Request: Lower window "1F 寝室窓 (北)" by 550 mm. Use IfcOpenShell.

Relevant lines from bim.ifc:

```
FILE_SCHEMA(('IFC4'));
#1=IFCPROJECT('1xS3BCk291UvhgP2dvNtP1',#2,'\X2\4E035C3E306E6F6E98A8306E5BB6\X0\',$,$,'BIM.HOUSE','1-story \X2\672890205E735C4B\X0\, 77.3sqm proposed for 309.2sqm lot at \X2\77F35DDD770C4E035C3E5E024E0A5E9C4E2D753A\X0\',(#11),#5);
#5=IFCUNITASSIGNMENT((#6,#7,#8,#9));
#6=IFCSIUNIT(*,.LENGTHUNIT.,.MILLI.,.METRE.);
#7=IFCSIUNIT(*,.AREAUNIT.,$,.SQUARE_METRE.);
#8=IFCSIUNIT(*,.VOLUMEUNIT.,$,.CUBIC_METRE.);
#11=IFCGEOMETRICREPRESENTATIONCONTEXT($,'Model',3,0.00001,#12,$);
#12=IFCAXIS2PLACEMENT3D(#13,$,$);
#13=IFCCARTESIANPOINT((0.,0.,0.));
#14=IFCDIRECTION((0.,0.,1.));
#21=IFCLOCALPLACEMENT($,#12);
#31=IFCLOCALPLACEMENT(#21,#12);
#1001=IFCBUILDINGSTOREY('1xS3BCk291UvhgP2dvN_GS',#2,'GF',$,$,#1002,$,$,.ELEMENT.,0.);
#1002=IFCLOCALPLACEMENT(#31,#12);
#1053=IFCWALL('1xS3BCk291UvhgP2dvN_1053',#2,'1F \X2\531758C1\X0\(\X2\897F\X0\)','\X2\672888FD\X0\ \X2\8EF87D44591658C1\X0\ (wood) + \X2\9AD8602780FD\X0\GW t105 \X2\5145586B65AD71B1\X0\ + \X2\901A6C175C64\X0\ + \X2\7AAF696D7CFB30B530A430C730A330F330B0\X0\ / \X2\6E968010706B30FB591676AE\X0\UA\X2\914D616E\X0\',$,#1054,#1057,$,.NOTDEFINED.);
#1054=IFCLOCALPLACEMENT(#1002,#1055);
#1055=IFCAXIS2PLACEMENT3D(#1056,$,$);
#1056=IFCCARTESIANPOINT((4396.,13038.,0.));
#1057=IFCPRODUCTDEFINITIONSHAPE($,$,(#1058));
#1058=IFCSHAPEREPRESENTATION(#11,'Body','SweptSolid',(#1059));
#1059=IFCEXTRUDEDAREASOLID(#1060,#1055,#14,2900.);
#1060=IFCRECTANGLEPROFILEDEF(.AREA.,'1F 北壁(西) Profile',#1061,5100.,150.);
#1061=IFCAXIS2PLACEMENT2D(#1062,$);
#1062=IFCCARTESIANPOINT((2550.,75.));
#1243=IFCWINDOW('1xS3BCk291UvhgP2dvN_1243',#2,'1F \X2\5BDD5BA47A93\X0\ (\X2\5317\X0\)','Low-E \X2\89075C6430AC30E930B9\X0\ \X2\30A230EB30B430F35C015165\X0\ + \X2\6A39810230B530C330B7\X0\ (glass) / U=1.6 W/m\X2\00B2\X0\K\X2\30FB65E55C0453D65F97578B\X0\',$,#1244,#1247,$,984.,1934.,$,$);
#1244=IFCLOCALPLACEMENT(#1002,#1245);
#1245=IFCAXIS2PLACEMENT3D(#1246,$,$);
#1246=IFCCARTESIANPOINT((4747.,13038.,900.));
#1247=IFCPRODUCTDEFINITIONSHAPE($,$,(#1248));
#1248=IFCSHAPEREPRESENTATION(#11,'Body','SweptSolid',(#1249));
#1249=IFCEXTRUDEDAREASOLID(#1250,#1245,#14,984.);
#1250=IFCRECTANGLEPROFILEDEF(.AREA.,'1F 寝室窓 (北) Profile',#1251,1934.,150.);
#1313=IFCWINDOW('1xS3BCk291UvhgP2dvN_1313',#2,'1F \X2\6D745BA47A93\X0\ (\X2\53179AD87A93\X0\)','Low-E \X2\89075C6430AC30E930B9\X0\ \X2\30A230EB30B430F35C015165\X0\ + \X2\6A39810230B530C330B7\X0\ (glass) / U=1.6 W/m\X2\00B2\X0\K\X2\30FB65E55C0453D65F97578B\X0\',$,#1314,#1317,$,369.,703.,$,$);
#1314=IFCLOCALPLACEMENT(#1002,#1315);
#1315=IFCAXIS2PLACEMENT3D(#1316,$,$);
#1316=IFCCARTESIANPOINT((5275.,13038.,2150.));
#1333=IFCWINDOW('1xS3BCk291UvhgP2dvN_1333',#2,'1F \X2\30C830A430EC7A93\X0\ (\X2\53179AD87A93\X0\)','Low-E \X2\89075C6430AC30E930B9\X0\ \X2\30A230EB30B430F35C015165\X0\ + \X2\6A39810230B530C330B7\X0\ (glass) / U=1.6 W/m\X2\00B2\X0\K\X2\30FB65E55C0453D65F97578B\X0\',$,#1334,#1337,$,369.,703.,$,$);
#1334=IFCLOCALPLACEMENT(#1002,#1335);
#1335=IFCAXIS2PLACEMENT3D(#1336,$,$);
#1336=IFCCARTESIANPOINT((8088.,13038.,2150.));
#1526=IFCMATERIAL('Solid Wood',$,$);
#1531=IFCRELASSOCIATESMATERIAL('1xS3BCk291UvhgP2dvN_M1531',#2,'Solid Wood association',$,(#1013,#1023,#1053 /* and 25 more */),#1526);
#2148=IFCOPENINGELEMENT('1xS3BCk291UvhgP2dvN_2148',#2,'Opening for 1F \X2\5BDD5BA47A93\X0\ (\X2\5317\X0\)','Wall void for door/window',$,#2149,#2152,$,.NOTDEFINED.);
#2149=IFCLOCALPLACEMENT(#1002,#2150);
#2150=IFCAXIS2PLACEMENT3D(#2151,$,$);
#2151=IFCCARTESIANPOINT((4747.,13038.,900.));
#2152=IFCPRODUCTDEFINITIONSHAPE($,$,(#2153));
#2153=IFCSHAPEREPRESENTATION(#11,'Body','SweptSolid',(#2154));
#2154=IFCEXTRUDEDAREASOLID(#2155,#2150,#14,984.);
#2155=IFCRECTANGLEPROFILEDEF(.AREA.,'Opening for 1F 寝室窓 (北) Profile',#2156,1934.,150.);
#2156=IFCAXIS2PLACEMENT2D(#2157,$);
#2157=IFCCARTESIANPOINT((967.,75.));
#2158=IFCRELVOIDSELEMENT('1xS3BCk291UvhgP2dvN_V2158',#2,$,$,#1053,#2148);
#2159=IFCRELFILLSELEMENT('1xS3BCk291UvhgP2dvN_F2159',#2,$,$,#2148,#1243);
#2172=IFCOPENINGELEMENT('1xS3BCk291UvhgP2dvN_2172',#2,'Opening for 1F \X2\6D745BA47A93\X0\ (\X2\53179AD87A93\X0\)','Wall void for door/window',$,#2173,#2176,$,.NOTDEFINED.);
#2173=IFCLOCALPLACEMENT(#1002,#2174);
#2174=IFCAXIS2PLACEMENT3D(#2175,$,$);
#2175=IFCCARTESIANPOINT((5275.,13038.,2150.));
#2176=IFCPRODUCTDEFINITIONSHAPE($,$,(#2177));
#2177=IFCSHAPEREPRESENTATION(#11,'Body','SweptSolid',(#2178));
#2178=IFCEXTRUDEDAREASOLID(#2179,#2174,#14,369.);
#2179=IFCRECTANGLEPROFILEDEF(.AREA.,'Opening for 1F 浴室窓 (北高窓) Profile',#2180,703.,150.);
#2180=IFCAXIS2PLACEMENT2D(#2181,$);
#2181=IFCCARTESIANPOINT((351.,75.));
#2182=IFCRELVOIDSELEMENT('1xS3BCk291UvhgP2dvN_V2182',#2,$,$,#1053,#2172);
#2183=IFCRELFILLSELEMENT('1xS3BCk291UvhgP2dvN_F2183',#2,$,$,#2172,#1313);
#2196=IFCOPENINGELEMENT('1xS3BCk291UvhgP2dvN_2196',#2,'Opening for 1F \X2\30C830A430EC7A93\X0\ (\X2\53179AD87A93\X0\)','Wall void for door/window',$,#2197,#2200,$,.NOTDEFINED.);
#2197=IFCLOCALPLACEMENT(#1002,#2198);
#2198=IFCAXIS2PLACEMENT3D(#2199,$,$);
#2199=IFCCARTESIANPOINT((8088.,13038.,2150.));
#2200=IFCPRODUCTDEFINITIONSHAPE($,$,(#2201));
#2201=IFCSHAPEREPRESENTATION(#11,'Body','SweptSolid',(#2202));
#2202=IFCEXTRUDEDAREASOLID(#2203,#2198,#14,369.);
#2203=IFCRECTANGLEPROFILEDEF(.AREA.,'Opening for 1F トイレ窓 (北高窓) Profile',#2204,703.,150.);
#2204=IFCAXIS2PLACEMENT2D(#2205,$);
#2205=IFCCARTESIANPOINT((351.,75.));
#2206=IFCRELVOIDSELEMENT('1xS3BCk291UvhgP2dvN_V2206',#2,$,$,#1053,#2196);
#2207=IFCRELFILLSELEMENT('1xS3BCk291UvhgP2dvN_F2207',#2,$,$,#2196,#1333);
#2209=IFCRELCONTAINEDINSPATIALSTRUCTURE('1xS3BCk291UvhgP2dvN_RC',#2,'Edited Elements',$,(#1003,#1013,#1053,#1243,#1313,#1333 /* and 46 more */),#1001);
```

```python
import numpy as np
import ifcopenshell
import ifcopenshell.api.geometry
import ifcopenshell.util.placement
import ifcopenshell.util.unit

model = ifcopenshell.open("bim.ifc")
unit_scale = ifcopenshell.util.unit.calculate_unit_scale(model)

window = model.by_guid("1xS3BCk291UvhgP2dvN_1243")
opening = window.FillsVoids[0].RelatingOpeningElement
dz = -550.0

shift = np.array([0.0, 0.0, dz])
# The window is not placed relative to its opening, so move both.
for product in (opening, window):
    matrix = ifcopenshell.util.placement.get_local_placement(product.ObjectPlacement)
    matrix[:3, 3] += shift
    ifcopenshell.api.geometry.edit_object_placement(model, product=product, matrix=matrix, is_si=False)

print(f"moved by {dz * unit_scale:+.3f} m")

model.write("bim-out.ifc")
```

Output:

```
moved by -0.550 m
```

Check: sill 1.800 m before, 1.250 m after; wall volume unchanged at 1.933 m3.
